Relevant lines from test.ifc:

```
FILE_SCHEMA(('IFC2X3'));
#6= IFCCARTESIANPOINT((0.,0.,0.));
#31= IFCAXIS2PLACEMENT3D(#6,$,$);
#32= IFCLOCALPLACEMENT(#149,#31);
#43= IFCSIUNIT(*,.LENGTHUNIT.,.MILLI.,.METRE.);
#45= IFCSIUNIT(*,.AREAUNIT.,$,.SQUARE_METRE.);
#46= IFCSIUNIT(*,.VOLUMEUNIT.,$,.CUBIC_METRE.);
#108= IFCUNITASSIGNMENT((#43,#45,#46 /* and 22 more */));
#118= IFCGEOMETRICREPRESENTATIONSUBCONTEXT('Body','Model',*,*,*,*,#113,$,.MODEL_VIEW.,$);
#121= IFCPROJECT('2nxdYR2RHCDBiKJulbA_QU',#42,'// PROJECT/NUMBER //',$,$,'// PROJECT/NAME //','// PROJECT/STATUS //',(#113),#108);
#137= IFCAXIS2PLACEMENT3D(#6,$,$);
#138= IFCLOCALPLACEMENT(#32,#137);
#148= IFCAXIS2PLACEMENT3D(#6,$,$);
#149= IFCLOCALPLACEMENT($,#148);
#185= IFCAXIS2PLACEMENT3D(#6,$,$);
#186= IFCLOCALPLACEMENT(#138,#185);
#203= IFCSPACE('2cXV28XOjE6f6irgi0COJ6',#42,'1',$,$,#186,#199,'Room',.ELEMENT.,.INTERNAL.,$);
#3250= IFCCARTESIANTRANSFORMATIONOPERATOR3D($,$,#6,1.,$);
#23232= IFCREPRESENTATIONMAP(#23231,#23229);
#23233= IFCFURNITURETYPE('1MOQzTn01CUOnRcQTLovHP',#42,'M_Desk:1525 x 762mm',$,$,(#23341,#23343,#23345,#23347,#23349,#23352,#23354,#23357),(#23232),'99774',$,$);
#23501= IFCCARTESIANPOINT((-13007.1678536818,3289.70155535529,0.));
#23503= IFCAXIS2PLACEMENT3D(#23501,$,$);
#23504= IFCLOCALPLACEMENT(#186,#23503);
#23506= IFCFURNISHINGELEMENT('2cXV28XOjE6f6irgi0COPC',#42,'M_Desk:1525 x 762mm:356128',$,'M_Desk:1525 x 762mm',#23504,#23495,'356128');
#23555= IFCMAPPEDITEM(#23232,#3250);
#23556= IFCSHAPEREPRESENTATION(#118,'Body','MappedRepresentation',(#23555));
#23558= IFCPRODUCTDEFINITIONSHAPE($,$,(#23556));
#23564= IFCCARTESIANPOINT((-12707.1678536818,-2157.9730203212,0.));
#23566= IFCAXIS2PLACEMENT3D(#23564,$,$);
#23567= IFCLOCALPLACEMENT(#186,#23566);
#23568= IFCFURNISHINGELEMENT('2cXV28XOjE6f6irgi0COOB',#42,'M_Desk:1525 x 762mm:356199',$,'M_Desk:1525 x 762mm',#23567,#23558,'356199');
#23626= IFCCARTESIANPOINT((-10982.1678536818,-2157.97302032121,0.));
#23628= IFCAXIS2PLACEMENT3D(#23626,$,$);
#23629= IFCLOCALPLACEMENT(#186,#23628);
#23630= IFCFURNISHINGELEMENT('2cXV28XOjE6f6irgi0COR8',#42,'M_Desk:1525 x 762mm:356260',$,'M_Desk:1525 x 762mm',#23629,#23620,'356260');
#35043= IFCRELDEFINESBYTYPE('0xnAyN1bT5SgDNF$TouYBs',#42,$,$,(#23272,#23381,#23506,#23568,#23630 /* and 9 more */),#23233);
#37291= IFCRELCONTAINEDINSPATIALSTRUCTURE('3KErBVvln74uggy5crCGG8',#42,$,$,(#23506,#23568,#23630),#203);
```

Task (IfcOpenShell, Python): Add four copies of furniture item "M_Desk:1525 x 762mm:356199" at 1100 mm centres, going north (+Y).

```python
import numpy as np
import ifcopenshell
import ifcopenshell.api.geometry
import ifcopenshell.api.root
import ifcopenshell.util.element
import ifcopenshell.util.placement
import ifcopenshell.util.unit

model = ifcopenshell.open("test.ifc")
unit_scale = ifcopenshell.util.unit.calculate_unit_scale(model)


def reuse_history(source, copy):
    """copy_class also copies each property set's owner history, people and application; keep the originals."""
    for rel in copy.IsDefinedBy:
        if rel.is_a("IfcRelDefinesByProperties") and (history := rel.RelatingPropertyDefinition.OwnerHistory):
            rel.RelatingPropertyDefinition.OwnerHistory = source.OwnerHistory
            ifcopenshell.util.element.remove_deep2(model, history)


source = model.by_guid("2cXV28XOjE6f6irgi0COOB")
base = ifcopenshell.util.placement.get_local_placement(source.ObjectPlacement)
step = np.array([0.0, 1.0, 0.0]) * 1.1 / unit_scale

for i in range(1, 5):
    copy = ifcopenshell.api.root.copy_class(model, product=source)
    copy.Representation = ifcopenshell.util.element.copy_deep(
        model, source.Representation, exclude=["IfcGeometricRepresentationContext", "IfcRepresentationMap"]
    )
    copy.Name = "M_Desk:1525 x 762mm"
    copy.Tag = None
    reuse_history(source, copy)
    matrix = base.copy()
    matrix[:3, 3] += i * step
    print("added at", matrix[:3, 3].round(3) + 0.0)
    ifcopenshell.api.geometry.edit_object_placement(model, product=copy, matrix=matrix, is_si=False)

model.write("test_edited.ifc")
```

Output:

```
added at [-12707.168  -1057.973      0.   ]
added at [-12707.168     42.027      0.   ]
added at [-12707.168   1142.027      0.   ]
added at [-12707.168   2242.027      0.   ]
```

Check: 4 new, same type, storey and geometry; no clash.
